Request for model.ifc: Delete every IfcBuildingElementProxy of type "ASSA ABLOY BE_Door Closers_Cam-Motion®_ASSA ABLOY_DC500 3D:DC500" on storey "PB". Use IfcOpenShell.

First a look at what the model holds.

```python
import ifcopenshell
import ifcopenshell.util.element

model = ifcopenshell.open("model.ifc")
print(model.schema)
storey = next(s for s in model.by_type("IfcBuildingStorey") if s.Name == "PB")
proxies = [e for e in ifcopenshell.util.element.get_decomposition(storey) if e.is_a("IfcBuildingElementProxy")]
seen = {}
for e in proxies:
    element_type = ifcopenshell.util.element.get_type(e)
    name = element_type.Name if element_type not in (None, e) else None
    seen[name] = seen.get(name, 0) + 1
for name, count in sorted(seen.items(), key=str):
    print(count, "x", name)
```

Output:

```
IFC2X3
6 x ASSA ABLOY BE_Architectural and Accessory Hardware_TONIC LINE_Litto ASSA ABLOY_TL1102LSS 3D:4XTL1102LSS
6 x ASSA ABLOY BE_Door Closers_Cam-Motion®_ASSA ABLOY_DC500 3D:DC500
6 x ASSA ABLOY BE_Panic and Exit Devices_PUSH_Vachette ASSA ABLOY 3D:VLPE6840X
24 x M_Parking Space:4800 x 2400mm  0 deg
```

```python
import ifcopenshell
import ifcopenshell.api.root
import ifcopenshell.util.element

model = ifcopenshell.open("model.ifc")

storey = next(s for s in model.by_type("IfcBuildingStorey") if s.Name == "PB")
proxies = [e for e in ifcopenshell.util.element.get_decomposition(storey) if e.is_a("IfcBuildingElementProxy")]
targets = [e for e in proxies if (t := ifcopenshell.util.element.get_type(e)) not in (None, e) and t.Name == "ASSA ABLOY BE_Door Closers_Cam-Motion®_ASSA ABLOY_DC500 3D:DC500"]

for e in targets:
    ifcopenshell.api.root.remove_product(model, product=e)
print(len(targets), "removed")

model.write("model-out.ifc")
```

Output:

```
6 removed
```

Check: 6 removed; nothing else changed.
